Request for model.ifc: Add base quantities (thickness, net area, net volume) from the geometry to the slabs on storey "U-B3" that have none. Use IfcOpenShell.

First a look at what the model holds.

```python
import ifcopenshell
import ifcopenshell.util.element
import ifcopenshell.util.unit

model = ifcopenshell.open("model.ifc")
print(model.schema)
for unit_type in ("LENGTHUNIT", "AREAUNIT", "VOLUMEUNIT"):
    print(unit_type, ifcopenshell.util.unit.calculate_unit_scale(model, unit_type))
storey = next(s for s in model.by_type("IfcBuildingStorey") if s.Name == "U-B3")
slabs = [e for e in ifcopenshell.util.element.get_decomposition(storey) if e.is_a("IfcSlab")]
for e in sorted(slabs, key=lambda e: e.id()):
    print(e.id(), e.is_a(), e.Name, list(ifcopenshell.util.element.get_psets(e, qtos_only=True)), sep=" | ")
```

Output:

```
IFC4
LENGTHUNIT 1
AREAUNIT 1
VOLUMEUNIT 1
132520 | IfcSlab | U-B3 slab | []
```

```python
import ifcopenshell
import ifcopenshell.api.pset
import ifcopenshell.geom
import ifcopenshell.util.element
import ifcopenshell.util.shape
import ifcopenshell.util.unit

model = ifcopenshell.open("model.ifc")
unit_scale = ifcopenshell.util.unit.calculate_unit_scale(model)
area_scale = ifcopenshell.util.unit.calculate_unit_scale(model, "AREAUNIT")
volume_scale = ifcopenshell.util.unit.calculate_unit_scale(model, "VOLUMEUNIT")
settings = ifcopenshell.geom.settings()

storey = next(s for s in model.by_type("IfcBuildingStorey") if s.Name == "U-B3")
slabs = [e for e in ifcopenshell.util.element.get_decomposition(storey) if e.is_a("IfcSlab")]

for e in sorted(slabs, key=lambda e: e.id()):
    if ifcopenshell.util.element.get_psets(e, qtos_only=True, should_inherit=False):
        continue
    # Geometry comes back in metres, in the element's own axes.
    shape = ifcopenshell.geom.create_shape(settings, e)
    values = {
        "Width": ifcopenshell.util.shape.get_z(shape.geometry) / unit_scale,
        "NetArea": ifcopenshell.util.shape.get_footprint_area(shape.geometry) / area_scale,
        "NetVolume": ifcopenshell.util.shape.get_volume(shape.geometry) / volume_scale,
    }
    qto = ifcopenshell.api.pset.add_qto(model, product=e, name="Qto_SlabBaseQuantities")
    ifcopenshell.api.pset.edit_qto(model, qto=qto, properties=values)
    print(e.id(), {k: round(v, 3) for k, v in values.items()})

model.write("model-out.ifc")
```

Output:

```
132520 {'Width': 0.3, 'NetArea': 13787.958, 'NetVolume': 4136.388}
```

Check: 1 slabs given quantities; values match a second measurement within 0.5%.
